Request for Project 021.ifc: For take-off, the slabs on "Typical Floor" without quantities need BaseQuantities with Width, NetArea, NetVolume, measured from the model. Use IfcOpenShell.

First a look at what the model holds.

```python
import ifcopenshell
import ifcopenshell.util.element
import ifcopenshell.util.unit

model = ifcopenshell.open("Project 021.ifc")
print(model.schema)
for unit_type in ("LENGTHUNIT", "AREAUNIT", "VOLUMEUNIT"):
    print(unit_type, ifcopenshell.util.unit.calculate_unit_scale(model, unit_type))
storey = next(s for s in model.by_type("IfcBuildingStorey") if s.Name == "Typical Floor")
slabs = [e for e in ifcopenshell.util.element.get_decomposition(storey) if e.is_a("IfcSlab")]
for e in sorted(slabs, key=lambda e: e.id()):
    print(e.id(), e.is_a(), e.Name, list(ifcopenshell.util.element.get_psets(e, qtos_only=True)), sep=" | ")
```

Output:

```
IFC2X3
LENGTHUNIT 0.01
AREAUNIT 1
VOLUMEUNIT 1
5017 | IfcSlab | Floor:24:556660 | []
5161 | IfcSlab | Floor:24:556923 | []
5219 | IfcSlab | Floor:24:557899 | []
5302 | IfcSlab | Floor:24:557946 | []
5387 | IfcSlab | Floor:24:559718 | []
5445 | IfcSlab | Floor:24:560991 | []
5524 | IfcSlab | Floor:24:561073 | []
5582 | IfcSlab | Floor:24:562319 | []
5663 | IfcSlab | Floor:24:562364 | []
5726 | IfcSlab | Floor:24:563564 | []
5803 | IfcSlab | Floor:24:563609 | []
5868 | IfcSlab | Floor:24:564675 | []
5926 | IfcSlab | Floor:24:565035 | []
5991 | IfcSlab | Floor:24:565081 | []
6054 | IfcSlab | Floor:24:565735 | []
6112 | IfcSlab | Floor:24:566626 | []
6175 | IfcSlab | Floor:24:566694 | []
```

```python
import ifcopenshell
import ifcopenshell.api.pset
import ifcopenshell.geom
import ifcopenshell.util.element
import ifcopenshell.util.shape
import ifcopenshell.util.unit

model = ifcopenshell.open("Project 021.ifc")
unit_scale = ifcopenshell.util.unit.calculate_unit_scale(model)
area_scale = ifcopenshell.util.unit.calculate_unit_scale(model, "AREAUNIT")
volume_scale = ifcopenshell.util.unit.calculate_unit_scale(model, "VOLUMEUNIT")
settings = ifcopenshell.geom.settings()

storey = next(s for s in model.by_type("IfcBuildingStorey") if s.Name == "Typical Floor")
slabs = [e for e in ifcopenshell.util.element.get_decomposition(storey) if e.is_a("IfcSlab")]

for e in sorted(slabs, key=lambda e: e.id()):
    if ifcopenshell.util.element.get_psets(e, qtos_only=True, should_inherit=False):
        continue
    # Geometry comes back in metres, in the element's own axes.
    shape = ifcopenshell.geom.create_shape(settings, e)
    values = {
        "Width": ifcopenshell.util.shape.get_z(shape.geometry) / unit_scale,
        "NetArea": ifcopenshell.util.shape.get_footprint_area(shape.geometry) / area_scale,
        "NetVolume": ifcopenshell.util.shape.get_volume(shape.geometry) / volume_scale,
    }
    qto = ifcopenshell.api.pset.add_qto(model, product=e, name="BaseQuantities")
    ifcopenshell.api.pset.edit_qto(model, qto=qto, properties=values)
    print(e.id(), {k: round(v, 3) for k, v in values.items()})

model.write("Project 021-out.ifc")
```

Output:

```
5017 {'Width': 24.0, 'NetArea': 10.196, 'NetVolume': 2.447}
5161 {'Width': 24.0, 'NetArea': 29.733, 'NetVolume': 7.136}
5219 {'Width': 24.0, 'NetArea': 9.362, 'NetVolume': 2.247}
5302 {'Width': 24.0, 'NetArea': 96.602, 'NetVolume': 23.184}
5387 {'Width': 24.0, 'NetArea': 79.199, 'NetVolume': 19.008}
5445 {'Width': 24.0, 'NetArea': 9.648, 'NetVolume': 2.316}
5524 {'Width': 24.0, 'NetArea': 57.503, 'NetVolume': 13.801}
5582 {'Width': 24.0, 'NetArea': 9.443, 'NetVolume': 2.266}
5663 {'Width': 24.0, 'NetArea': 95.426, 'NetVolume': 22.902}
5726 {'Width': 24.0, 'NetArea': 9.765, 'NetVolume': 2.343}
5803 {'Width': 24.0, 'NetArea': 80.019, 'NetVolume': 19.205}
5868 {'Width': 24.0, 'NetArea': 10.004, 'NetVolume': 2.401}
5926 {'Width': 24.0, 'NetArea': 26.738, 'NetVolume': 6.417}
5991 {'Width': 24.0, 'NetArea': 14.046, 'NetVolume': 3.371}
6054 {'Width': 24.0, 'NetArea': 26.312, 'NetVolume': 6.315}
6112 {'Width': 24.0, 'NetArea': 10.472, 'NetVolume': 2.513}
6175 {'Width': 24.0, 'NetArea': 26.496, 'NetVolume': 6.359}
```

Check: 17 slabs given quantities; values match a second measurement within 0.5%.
